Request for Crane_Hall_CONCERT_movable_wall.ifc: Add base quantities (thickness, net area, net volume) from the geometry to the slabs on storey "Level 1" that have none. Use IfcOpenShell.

First a look at what the model holds.

```python
import ifcopenshell
import ifcopenshell.util.element
import ifcopenshell.util.unit

model = ifcopenshell.open("Crane_Hall_CONCERT_movable_wall.ifc")
print(model.schema)
for unit_type in ("LENGTHUNIT", "AREAUNIT", "VOLUMEUNIT"):
    print(unit_type, ifcopenshell.util.unit.calculate_unit_scale(model, unit_type))
storey = next(s for s in model.by_type("IfcBuildingStorey") if s.Name == "Level 1")
slabs = [e for e in ifcopenshell.util.element.get_decomposition(storey) if e.is_a("IfcSlab")]
for e in sorted(slabs, key=lambda e: e.id()):
    print(e.id(), e.is_a(), e.Name, list(ifcopenshell.util.element.get_psets(e, qtos_only=True)), sep=" | ")
```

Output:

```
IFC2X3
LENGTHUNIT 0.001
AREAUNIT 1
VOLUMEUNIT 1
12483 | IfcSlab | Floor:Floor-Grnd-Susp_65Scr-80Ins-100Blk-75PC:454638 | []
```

```python
import ifcopenshell
import ifcopenshell.api.pset
import ifcopenshell.geom
import ifcopenshell.util.element
import ifcopenshell.util.shape
import ifcopenshell.util.unit

model = ifcopenshell.open("Crane_Hall_CONCERT_movable_wall.ifc")
unit_scale = ifcopenshell.util.unit.calculate_unit_scale(model)
area_scale = ifcopenshell.util.unit.calculate_unit_scale(model, "AREAUNIT")
volume_scale = ifcopenshell.util.unit.calculate_unit_scale(model, "VOLUMEUNIT")
settings = ifcopenshell.geom.settings()

storey = next(s for s in model.by_type("IfcBuildingStorey") if s.Name == "Level 1")
slabs = [e for e in ifcopenshell.util.element.get_decomposition(storey) if e.is_a("IfcSlab")]

for e in sorted(slabs, key=lambda e: e.id()):
    if ifcopenshell.util.element.get_psets(e, qtos_only=True, should_inherit=False):
        continue
    # Geometry comes back in metres, in the element's own axes.
    shape = ifcopenshell.geom.create_shape(settings, e)
    values = {
        "Width": ifcopenshell.util.shape.get_z(shape.geometry) / unit_scale,
        "NetArea": ifcopenshell.util.shape.get_footprint_area(shape.geometry) / area_scale,
        "NetVolume": ifcopenshell.util.shape.get_volume(shape.geometry) / volume_scale,
    }
    qto = ifcopenshell.api.pset.add_qto(model, product=e, name="BaseQuantities")
    ifcopenshell.api.pset.edit_qto(model, qto=qto, properties=values)
    print(e.id(), {k: round(v, 3) for k, v in values.items()})

model.write("Crane_Hall_CONCERT_movable_wall-out.ifc")
```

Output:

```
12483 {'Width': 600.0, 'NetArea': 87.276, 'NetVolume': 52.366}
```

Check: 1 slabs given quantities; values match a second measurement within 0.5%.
